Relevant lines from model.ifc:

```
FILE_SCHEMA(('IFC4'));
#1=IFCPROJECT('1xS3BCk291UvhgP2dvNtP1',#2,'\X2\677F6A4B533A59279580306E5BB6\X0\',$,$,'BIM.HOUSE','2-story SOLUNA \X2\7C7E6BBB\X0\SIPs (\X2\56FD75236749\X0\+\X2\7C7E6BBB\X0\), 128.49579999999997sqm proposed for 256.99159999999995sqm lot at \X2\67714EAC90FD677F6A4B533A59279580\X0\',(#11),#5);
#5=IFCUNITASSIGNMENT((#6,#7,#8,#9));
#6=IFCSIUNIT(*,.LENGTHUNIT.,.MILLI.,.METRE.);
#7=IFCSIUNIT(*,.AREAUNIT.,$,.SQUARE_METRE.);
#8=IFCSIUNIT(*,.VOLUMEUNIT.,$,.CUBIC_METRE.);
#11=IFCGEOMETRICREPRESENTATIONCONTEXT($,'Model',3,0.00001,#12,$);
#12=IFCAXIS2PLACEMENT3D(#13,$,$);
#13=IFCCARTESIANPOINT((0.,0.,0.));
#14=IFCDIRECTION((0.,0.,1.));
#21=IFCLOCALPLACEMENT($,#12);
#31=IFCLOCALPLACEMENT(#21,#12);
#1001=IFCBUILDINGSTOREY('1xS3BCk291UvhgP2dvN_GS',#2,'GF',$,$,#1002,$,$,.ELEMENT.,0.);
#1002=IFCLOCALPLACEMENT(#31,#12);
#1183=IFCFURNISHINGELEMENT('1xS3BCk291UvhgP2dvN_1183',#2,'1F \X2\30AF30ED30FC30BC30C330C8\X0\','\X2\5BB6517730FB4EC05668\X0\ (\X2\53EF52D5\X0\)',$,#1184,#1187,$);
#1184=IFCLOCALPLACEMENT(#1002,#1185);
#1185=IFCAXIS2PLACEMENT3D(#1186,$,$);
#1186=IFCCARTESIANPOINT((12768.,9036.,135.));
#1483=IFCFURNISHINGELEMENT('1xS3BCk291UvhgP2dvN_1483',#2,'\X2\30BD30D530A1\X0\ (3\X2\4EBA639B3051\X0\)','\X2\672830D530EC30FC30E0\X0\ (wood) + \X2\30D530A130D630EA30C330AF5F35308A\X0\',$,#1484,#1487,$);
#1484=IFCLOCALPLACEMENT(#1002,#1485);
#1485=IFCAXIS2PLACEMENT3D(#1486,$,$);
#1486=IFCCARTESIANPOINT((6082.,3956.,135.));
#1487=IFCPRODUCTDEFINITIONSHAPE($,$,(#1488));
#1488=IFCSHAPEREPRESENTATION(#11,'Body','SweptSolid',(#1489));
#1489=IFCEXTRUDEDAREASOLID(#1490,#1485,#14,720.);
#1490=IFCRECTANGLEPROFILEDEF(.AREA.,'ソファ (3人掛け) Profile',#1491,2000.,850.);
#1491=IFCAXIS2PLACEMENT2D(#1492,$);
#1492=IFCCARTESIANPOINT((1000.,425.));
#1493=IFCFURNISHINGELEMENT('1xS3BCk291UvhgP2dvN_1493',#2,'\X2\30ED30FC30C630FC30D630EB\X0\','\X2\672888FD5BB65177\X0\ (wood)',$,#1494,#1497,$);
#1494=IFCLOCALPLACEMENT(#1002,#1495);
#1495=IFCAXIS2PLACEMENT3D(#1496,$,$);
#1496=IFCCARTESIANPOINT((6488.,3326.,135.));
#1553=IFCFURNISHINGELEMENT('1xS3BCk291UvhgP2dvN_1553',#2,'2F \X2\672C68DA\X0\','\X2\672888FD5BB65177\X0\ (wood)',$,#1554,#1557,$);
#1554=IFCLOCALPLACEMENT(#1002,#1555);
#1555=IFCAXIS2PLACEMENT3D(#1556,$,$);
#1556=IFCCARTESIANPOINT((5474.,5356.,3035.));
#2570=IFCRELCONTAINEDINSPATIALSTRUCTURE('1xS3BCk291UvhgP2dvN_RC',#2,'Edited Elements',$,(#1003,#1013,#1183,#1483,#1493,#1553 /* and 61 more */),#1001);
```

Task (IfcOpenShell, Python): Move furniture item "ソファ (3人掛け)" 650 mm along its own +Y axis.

```python
import ifcopenshell
import ifcopenshell.api.geometry
import ifcopenshell.util.placement
import ifcopenshell.util.unit

model = ifcopenshell.open("model.ifc")
unit_scale = ifcopenshell.util.unit.calculate_unit_scale(model)

item = model.by_id(1483)
matrix = ifcopenshell.util.placement.get_local_placement(item.ObjectPlacement)
matrix[:3, 3] += matrix[:3, 1] * 0.65 / unit_scale
ifcopenshell.api.geometry.edit_object_placement(model, product=item, matrix=matrix, is_si=False)

print(ifcopenshell.util.placement.get_local_placement(item.ObjectPlacement).round(3) + 0.0)

model.write("model_v2.ifc")
```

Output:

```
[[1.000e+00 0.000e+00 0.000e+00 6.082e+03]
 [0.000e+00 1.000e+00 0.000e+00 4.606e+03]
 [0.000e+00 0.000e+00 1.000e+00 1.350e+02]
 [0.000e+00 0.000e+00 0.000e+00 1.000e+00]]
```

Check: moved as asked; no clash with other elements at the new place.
